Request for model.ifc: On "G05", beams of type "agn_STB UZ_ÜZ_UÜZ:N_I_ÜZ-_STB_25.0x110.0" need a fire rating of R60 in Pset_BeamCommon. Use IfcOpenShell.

First a look at what the model holds.

```python
import ifcopenshell
import ifcopenshell.util.element

model = ifcopenshell.open("model.ifc")
print(model.schema)
storey = next(s for s in model.by_type("IfcBuildingStorey") if s.Name == "G05")
beams = [e for e in ifcopenshell.util.element.get_decomposition(storey) if e.is_a("IfcBeam")]
seen = {}
for e in beams:
    element_type = ifcopenshell.util.element.get_type(e)
    key = (element_type.Name if element_type != e and element_type else None, ifcopenshell.util.element.get_pset(e, "Pset_BeamCommon", "FireRating"))
    seen[key] = seen.get(key, 0) + 1
for (name, value), count in sorted(seen.items(), key=str):
    print(count, "x", name, "|", value)
```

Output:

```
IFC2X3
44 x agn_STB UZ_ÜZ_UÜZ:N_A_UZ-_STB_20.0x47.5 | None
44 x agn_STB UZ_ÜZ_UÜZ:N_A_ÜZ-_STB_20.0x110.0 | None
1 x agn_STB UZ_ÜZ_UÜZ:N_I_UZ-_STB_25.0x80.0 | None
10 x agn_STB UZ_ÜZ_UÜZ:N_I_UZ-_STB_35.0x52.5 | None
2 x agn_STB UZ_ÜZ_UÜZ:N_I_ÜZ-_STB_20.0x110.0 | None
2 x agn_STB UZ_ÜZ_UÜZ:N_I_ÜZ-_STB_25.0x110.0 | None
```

```python
import ifcopenshell
import ifcopenshell.api.pset
import ifcopenshell.util.element

model = ifcopenshell.open("model.ifc")

storey = next(s for s in model.by_type("IfcBuildingStorey") if s.Name == "G05")
beams = [e for e in ifcopenshell.util.element.get_decomposition(storey) if e.is_a("IfcBeam")]

count = 0
for e in beams:
    element_type = ifcopenshell.util.element.get_type(e)
    if element_type in (None, e) or element_type.Name != "agn_STB UZ_ÜZ_UÜZ:N_I_ÜZ-_STB_25.0x110.0":
        continue
    found = ifcopenshell.util.element.get_pset(e, "Pset_BeamCommon", should_inherit=False)
    if found:
        pset = model.by_id(found["id"])
        if len(ifcopenshell.util.element.get_elements_by_pset(pset)) > 1:
            pset = ifcopenshell.api.pset.unshare_pset(model, products=[e], pset=pset)[0]
    else:
        pset = ifcopenshell.api.pset.add_pset(model, product=e, name="Pset_BeamCommon")
    ifcopenshell.api.pset.edit_pset(model, pset=pset, properties={"FireRating": "R60"})
    count += 1

print(count, "beams updated")

model.write("model_updated.ifc")
```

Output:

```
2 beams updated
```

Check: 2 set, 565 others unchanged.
